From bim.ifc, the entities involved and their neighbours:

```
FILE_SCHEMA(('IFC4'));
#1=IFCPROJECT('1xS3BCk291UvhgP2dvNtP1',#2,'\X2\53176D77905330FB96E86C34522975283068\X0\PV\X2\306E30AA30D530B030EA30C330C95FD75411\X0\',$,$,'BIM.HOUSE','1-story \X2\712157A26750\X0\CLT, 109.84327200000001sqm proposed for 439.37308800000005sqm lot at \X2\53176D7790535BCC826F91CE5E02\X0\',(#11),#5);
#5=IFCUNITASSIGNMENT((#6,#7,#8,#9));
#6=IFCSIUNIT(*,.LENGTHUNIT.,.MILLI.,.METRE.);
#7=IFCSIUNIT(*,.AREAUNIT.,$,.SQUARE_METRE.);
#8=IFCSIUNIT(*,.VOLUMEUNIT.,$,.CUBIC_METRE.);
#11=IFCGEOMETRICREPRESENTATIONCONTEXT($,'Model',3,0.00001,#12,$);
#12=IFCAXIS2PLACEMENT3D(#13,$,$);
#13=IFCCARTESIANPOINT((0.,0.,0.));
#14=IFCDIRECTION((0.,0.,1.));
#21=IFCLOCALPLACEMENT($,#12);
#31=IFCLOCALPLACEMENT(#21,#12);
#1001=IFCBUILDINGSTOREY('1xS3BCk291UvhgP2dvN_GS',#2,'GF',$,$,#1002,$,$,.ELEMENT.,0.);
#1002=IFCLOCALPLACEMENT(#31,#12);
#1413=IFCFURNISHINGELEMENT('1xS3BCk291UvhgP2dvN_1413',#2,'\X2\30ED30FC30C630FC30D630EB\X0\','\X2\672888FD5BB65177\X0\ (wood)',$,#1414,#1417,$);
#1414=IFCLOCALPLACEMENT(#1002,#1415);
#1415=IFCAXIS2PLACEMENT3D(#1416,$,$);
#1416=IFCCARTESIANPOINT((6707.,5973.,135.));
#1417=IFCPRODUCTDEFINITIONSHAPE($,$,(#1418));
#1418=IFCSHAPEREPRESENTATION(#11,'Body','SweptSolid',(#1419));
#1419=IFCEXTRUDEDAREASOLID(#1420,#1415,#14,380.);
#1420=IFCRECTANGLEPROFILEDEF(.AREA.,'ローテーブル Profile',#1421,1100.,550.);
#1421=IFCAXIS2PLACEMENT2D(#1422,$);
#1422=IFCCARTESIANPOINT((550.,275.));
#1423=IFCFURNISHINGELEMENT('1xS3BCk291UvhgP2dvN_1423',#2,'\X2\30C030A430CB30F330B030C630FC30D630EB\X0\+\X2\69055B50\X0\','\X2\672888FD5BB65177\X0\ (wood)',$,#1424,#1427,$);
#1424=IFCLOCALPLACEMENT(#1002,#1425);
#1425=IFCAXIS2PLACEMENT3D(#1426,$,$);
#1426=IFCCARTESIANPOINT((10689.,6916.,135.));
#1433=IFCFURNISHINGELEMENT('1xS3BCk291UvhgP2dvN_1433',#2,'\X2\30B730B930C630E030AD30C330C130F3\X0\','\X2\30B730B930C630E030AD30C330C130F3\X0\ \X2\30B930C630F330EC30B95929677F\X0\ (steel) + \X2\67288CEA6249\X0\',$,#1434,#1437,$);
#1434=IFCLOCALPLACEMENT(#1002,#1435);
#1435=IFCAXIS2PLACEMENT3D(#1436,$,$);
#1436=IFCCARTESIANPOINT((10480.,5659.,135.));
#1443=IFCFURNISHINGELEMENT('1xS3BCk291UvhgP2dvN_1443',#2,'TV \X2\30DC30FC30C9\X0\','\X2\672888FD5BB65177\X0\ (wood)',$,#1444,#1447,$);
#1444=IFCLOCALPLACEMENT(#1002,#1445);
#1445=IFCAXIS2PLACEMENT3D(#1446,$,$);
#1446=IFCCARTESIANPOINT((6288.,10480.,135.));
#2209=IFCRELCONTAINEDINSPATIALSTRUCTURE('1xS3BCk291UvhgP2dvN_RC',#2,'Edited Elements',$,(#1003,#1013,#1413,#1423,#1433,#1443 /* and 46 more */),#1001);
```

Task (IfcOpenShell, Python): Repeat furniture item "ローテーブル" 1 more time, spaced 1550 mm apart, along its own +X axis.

```python
import ifcopenshell
import ifcopenshell.api.geometry
import ifcopenshell.api.root
import ifcopenshell.util.element
import ifcopenshell.util.placement
import ifcopenshell.util.unit

model = ifcopenshell.open("bim.ifc")
unit_scale = ifcopenshell.util.unit.calculate_unit_scale(model)


def reuse_history(source, copy):
    """copy_class also copies each property set's owner history, people and application; keep the originals."""
    for rel in copy.IsDefinedBy:
        if rel.is_a("IfcRelDefinesByProperties") and (history := rel.RelatingPropertyDefinition.OwnerHistory):
            rel.RelatingPropertyDefinition.OwnerHistory = source.OwnerHistory
            ifcopenshell.util.element.remove_deep2(model, history)


source = model.by_guid("1xS3BCk291UvhgP2dvN_1413")
base = ifcopenshell.util.placement.get_local_placement(source.ObjectPlacement)
step = base[:3, 0] * 1.55 / unit_scale

for i in range(1, 2):
    copy = ifcopenshell.api.root.copy_class(model, product=source)
    copy.Representation = ifcopenshell.util.element.copy_deep(
        model, source.Representation, exclude=["IfcGeometricRepresentationContext", "IfcRepresentationMap"]
    )
    reuse_history(source, copy)
    matrix = base.copy()
    matrix[:3, 3] += i * step
    print("added at", matrix[:3, 3].round(3) + 0.0)
    ifcopenshell.api.geometry.edit_object_placement(model, product=copy, matrix=matrix, is_si=False)

model.write("bim_v2.ifc")
```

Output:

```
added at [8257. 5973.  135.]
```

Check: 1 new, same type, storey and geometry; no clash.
